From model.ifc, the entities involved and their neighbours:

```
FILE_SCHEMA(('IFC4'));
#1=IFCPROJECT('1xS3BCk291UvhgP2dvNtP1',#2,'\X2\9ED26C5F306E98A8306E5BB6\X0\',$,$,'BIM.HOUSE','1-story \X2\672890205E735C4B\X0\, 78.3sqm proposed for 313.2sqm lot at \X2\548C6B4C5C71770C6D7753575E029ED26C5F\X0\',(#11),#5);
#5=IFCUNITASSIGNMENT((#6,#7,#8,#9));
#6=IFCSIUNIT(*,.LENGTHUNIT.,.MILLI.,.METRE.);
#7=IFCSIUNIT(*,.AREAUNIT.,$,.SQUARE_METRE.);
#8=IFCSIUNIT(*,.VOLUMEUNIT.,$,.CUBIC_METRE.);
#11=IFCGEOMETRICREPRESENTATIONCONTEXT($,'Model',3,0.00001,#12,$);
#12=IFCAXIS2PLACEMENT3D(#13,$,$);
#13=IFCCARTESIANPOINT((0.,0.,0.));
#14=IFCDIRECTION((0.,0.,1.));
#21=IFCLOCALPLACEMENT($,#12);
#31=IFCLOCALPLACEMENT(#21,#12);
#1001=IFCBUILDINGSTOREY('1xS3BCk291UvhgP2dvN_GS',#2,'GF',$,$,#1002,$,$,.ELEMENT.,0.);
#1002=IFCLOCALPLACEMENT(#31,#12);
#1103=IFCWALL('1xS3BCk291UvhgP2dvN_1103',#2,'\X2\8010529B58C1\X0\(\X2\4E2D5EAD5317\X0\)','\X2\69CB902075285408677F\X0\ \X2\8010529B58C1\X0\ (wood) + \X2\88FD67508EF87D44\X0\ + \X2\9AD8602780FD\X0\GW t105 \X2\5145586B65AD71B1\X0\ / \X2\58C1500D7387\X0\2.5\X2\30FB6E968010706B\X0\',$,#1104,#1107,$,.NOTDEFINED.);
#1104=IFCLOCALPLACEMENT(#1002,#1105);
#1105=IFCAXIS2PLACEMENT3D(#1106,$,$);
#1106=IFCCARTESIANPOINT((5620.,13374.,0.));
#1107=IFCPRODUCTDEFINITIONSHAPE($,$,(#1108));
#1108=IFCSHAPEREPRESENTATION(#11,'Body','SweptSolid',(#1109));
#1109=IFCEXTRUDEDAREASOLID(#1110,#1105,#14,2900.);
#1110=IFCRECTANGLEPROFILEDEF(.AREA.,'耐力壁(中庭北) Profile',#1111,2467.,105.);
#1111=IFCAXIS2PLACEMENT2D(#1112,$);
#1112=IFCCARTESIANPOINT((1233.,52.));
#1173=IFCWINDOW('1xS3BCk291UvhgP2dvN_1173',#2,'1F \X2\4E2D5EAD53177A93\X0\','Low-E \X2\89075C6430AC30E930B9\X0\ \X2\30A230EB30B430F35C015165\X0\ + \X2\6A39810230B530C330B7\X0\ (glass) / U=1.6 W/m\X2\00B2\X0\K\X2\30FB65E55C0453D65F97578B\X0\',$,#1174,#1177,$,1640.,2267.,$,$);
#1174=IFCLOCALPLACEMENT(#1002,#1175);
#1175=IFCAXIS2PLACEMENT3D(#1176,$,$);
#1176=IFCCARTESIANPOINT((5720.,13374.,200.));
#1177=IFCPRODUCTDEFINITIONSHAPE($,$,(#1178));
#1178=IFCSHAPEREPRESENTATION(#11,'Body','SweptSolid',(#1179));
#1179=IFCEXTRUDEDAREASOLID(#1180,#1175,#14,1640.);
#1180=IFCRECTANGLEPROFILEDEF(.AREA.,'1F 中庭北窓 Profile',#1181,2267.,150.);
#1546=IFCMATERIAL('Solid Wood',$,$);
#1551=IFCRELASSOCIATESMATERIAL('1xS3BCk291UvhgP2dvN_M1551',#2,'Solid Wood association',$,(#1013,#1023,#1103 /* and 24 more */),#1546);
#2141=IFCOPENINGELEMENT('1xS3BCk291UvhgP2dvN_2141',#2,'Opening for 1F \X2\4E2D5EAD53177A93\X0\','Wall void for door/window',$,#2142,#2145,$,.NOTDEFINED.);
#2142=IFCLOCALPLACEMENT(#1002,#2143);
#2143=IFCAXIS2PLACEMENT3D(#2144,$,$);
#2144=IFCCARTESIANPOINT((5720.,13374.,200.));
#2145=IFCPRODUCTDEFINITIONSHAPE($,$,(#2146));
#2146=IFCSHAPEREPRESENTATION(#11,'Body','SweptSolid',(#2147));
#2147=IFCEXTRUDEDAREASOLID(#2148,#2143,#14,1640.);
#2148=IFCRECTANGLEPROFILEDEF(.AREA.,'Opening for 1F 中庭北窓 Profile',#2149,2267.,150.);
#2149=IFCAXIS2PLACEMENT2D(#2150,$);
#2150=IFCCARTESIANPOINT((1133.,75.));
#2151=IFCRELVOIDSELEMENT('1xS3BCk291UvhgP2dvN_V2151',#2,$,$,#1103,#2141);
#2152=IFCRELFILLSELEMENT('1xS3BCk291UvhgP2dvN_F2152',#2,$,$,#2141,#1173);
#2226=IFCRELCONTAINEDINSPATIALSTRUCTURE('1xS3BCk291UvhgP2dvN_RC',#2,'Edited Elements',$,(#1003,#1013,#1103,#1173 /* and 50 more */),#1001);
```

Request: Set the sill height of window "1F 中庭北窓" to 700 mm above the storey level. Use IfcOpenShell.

```python
import numpy as np
import ifcopenshell
import ifcopenshell.api.geometry
import ifcopenshell.geom
import ifcopenshell.util.element
import ifcopenshell.util.placement
import ifcopenshell.util.shape
import ifcopenshell.util.unit

model = ifcopenshell.open("model.ifc")
unit_scale = ifcopenshell.util.unit.calculate_unit_scale(model)

window = model.by_guid("1xS3BCk291UvhgP2dvN_1173")
opening = window.FillsVoids[0].RelatingOpeningElement
storey = ifcopenshell.util.element.get_container(window, ifc_class="IfcBuildingStorey")
level = ifcopenshell.util.placement.get_local_placement(storey.ObjectPlacement)[2, 3]

# The opening's origin need not be at the sill, so measure its lowest point.
shape = ifcopenshell.geom.create_shape(ifcopenshell.geom.settings(), opening)
bottom = ifcopenshell.util.shape.get_shape_bottom_elevation(shape, shape.geometry) / unit_scale
dz = level + 700.0 - bottom

shift = np.array([0.0, 0.0, dz])
# The window is not placed relative to its opening, so move both.
for product in (opening, window):
    matrix = ifcopenshell.util.placement.get_local_placement(product.ObjectPlacement)
    matrix[:3, 3] += shift
    ifcopenshell.api.geometry.edit_object_placement(model, product=product, matrix=matrix, is_si=False)

print(f"moved by {dz * unit_scale:+.3f} m")

model.write("model_v2.ifc")
```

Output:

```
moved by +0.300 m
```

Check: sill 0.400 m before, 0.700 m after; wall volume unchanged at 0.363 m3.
